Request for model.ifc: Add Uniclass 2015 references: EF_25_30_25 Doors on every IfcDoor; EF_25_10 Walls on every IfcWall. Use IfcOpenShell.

First a look at what the model holds.

```python
import ifcopenshell

model = ifcopenshell.open("model.ifc")
print(model.schema)
print("classifications:", [c.Name for c in model.by_type("IfcClassification")])
for ifc_class in ("IfcDoor", "IfcRoof", "IfcStair", "IfcWall", "IfcWindow"):
    print(ifc_class, len(model.by_type(ifc_class)))
```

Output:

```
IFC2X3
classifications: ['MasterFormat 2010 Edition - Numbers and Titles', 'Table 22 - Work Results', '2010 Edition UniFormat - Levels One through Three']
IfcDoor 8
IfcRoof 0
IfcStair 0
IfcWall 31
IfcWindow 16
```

```python
import ifcopenshell
import ifcopenshell.api.classification

model = ifcopenshell.open("model.ifc")

# IFC2X3 requires Source and Edition and has no link from the project to the system.
system = model.create_entity("IfcClassification", Source="NBS", Edition="2015", Name="Uniclass 2015")

codes = {
    "IfcDoor": ("EF_25_30_25", "Doors"),
    "IfcWall": ("EF_25_10", "Walls"),
}
for ifc_class, (code, name) in codes.items():
    products = model.by_type(ifc_class)
    ifcopenshell.api.classification.add_reference(
        model, products=products, classification=system, identification=code, name=name
    )
    print(code, len(products))

model.write("model_updated.ifc")
```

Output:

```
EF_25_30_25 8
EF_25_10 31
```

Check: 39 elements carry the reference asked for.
